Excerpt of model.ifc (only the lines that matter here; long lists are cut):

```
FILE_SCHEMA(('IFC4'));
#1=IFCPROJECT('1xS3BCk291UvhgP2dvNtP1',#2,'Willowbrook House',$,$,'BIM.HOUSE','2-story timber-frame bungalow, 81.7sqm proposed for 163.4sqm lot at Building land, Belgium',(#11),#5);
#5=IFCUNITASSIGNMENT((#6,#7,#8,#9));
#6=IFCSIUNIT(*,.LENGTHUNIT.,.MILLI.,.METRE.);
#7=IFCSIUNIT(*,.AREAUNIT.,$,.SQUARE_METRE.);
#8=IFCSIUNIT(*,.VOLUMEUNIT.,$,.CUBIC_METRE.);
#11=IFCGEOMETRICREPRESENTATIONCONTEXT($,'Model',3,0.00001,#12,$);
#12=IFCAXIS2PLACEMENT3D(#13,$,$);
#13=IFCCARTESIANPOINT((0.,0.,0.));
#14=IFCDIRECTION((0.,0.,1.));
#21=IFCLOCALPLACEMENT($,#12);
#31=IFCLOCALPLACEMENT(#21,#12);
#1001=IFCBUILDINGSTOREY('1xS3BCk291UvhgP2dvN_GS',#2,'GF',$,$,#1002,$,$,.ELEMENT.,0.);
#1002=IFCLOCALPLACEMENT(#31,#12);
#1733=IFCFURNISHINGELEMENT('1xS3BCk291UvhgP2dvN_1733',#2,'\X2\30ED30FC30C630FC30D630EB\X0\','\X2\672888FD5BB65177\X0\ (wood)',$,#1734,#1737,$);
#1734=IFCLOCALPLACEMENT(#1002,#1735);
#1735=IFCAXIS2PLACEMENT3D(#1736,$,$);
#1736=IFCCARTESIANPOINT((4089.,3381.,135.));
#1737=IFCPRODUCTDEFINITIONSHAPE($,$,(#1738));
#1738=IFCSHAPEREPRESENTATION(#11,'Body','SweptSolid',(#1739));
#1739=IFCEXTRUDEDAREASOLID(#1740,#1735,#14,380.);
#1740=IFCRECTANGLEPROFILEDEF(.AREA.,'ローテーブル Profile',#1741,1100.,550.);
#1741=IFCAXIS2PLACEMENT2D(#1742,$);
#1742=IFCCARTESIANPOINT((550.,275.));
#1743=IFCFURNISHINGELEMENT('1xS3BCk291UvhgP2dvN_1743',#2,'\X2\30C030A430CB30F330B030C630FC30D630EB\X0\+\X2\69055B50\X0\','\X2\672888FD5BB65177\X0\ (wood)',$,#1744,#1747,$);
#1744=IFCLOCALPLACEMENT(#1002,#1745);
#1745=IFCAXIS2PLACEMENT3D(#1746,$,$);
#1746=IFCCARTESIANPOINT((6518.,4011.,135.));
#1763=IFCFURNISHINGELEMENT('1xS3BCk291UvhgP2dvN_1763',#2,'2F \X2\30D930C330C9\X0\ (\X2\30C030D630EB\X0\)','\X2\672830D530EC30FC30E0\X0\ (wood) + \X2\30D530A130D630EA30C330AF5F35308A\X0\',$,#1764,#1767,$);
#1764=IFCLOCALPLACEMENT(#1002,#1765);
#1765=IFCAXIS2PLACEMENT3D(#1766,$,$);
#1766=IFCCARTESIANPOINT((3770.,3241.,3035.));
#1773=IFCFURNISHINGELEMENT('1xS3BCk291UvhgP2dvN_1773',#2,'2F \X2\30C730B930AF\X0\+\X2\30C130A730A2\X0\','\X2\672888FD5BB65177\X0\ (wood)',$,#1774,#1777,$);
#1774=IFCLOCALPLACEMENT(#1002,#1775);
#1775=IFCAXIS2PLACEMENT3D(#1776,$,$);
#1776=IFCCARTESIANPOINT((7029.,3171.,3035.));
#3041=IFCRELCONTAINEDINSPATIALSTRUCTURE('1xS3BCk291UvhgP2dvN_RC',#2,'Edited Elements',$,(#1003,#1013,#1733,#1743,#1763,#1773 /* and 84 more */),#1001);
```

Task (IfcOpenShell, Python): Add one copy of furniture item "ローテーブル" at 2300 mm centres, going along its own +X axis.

```python
import ifcopenshell
import ifcopenshell.api.geometry
import ifcopenshell.api.root
import ifcopenshell.util.element
import ifcopenshell.util.placement

model = ifcopenshell.open("model.ifc")


def reuse_history(source, copy):
    """copy_class also copies each property set's owner history, people and application; keep the originals."""
    for rel in copy.IsDefinedBy:
        if rel.is_a("IfcRelDefinesByProperties") and (history := rel.RelatingPropertyDefinition.OwnerHistory):
            rel.RelatingPropertyDefinition.OwnerHistory = source.OwnerHistory
            ifcopenshell.util.element.remove_deep2(model, history)


source = model.by_id(1733)
base = ifcopenshell.util.placement.get_local_placement(source.ObjectPlacement)
step = base[:3, 0] * 2300.0

for i in range(1, 2):
    copy = ifcopenshell.api.root.copy_class(model, product=source)
    copy.Representation = ifcopenshell.util.element.copy_deep(
        model, source.Representation, exclude=["IfcGeometricRepresentationContext", "IfcRepresentationMap"]
    )
    reuse_history(source, copy)
    matrix = base.copy()
    matrix[:3, 3] += i * step
    print("added at", matrix[:3, 3].round(3) + 0.0)
    ifcopenshell.api.geometry.edit_object_placement(model, product=copy, matrix=matrix, is_si=False)

model.write("model_updated.ifc")
```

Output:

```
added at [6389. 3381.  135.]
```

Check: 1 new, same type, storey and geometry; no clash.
